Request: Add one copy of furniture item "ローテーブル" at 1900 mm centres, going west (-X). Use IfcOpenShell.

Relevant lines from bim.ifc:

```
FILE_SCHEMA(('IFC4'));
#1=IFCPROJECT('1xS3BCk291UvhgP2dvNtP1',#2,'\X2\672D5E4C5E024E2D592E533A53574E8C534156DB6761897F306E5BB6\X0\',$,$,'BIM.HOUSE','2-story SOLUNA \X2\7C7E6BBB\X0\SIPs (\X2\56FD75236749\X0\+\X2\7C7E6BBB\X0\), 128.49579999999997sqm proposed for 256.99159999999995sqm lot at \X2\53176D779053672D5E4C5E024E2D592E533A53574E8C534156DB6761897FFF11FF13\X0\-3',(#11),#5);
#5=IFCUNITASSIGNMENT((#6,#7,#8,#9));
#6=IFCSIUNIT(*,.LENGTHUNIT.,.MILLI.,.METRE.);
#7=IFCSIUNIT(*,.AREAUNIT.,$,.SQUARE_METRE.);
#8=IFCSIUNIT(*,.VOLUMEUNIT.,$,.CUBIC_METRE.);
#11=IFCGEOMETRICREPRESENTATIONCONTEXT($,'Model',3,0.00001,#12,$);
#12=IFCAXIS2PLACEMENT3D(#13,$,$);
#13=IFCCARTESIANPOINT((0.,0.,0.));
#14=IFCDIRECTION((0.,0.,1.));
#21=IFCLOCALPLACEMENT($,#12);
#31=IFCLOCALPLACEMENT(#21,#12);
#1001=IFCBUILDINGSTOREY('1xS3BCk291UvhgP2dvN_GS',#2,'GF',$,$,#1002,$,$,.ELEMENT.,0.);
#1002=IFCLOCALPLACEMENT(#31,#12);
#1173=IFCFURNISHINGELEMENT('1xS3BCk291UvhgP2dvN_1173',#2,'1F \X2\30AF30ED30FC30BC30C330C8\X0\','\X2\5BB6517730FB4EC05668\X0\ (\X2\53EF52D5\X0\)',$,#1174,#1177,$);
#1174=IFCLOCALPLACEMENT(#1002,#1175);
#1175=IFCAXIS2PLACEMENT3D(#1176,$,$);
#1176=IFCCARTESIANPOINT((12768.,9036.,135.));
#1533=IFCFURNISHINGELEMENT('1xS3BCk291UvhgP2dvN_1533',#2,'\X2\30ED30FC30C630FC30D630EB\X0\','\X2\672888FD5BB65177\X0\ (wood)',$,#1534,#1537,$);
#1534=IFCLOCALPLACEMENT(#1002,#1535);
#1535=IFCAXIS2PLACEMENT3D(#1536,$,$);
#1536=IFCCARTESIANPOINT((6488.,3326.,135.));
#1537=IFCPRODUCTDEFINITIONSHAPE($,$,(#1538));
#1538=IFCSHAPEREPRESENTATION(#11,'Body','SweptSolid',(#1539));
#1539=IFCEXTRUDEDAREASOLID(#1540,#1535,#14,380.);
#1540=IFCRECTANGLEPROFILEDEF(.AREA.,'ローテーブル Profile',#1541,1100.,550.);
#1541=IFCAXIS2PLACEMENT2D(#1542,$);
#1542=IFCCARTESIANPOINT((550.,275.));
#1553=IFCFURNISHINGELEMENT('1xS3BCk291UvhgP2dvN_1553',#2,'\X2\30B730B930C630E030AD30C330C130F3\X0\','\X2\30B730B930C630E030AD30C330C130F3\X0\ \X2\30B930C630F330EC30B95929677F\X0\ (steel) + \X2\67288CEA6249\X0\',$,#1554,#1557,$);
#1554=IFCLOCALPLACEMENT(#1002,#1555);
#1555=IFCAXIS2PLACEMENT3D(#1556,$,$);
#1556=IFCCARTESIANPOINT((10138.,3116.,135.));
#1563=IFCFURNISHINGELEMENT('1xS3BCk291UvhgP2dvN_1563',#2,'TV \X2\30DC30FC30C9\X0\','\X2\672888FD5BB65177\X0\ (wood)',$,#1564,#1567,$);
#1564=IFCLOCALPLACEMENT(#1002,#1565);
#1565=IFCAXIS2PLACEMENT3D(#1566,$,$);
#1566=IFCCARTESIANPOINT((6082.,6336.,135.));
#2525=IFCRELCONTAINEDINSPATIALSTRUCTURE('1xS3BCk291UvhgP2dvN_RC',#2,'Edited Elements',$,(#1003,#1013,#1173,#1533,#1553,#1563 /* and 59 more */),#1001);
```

```python
import numpy as np
import ifcopenshell
import ifcopenshell.api.geometry
import ifcopenshell.api.root
import ifcopenshell.util.element
import ifcopenshell.util.placement
import ifcopenshell.util.unit

model = ifcopenshell.open("bim.ifc")
unit_scale = ifcopenshell.util.unit.calculate_unit_scale(model)


def reuse_history(source, copy):
    """copy_class also copies each property set's owner history, people and application; keep the originals."""
    for rel in copy.IsDefinedBy:
        if rel.is_a("IfcRelDefinesByProperties") and (history := rel.RelatingPropertyDefinition.OwnerHistory):
            rel.RelatingPropertyDefinition.OwnerHistory = source.OwnerHistory
            ifcopenshell.util.element.remove_deep2(model, history)


source = model.by_guid("1xS3BCk291UvhgP2dvN_1533")
base = ifcopenshell.util.placement.get_local_placement(source.ObjectPlacement)
step = np.array([-1.0, 0.0, 0.0]) * 1.9 / unit_scale

for i in range(1, 2):
    copy = ifcopenshell.api.root.copy_class(model, product=source)
    copy.Representation = ifcopenshell.util.element.copy_deep(
        model, source.Representation, exclude=["IfcGeometricRepresentationContext", "IfcRepresentationMap"]
    )
    reuse_history(source, copy)
    matrix = base.copy()
    matrix[:3, 3] += i * step
    print("added at", matrix[:3, 3].round(3) + 0.0)
    ifcopenshell.api.geometry.edit_object_placement(model, product=copy, matrix=matrix, is_si=False)

model.write("bim-out.ifc")
```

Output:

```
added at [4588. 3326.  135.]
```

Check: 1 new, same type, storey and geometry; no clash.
